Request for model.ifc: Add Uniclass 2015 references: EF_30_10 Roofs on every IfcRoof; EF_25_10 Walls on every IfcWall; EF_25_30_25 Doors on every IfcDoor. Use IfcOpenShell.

First a look at what the model holds.

```python
import ifcopenshell

model = ifcopenshell.open("model.ifc")
print(model.schema)
print("classifications:", [c.Name for c in model.by_type("IfcClassification")])
for ifc_class in ("IfcDoor", "IfcRoof", "IfcStair", "IfcWall", "IfcWindow"):
    print(ifc_class, len(model.by_type(ifc_class)))
```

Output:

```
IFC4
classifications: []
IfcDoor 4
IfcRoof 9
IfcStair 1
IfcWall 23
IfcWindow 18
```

```python
import ifcopenshell
import ifcopenshell.api.classification

model = ifcopenshell.open("model.ifc")

system = ifcopenshell.api.classification.add_classification(model, classification="Uniclass 2015")

codes = {
    "IfcRoof": ("EF_30_10", "Roofs"),
    "IfcWall": ("EF_25_10", "Walls"),
    "IfcDoor": ("EF_25_30_25", "Doors"),
}
for ifc_class, (code, name) in codes.items():
    products = model.by_type(ifc_class)
    ifcopenshell.api.classification.add_reference(
        model, products=products, classification=system, identification=code, name=name
    )
    print(code, len(products))

model.write("model_rev.ifc")
```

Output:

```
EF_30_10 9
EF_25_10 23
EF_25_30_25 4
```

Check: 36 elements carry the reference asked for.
